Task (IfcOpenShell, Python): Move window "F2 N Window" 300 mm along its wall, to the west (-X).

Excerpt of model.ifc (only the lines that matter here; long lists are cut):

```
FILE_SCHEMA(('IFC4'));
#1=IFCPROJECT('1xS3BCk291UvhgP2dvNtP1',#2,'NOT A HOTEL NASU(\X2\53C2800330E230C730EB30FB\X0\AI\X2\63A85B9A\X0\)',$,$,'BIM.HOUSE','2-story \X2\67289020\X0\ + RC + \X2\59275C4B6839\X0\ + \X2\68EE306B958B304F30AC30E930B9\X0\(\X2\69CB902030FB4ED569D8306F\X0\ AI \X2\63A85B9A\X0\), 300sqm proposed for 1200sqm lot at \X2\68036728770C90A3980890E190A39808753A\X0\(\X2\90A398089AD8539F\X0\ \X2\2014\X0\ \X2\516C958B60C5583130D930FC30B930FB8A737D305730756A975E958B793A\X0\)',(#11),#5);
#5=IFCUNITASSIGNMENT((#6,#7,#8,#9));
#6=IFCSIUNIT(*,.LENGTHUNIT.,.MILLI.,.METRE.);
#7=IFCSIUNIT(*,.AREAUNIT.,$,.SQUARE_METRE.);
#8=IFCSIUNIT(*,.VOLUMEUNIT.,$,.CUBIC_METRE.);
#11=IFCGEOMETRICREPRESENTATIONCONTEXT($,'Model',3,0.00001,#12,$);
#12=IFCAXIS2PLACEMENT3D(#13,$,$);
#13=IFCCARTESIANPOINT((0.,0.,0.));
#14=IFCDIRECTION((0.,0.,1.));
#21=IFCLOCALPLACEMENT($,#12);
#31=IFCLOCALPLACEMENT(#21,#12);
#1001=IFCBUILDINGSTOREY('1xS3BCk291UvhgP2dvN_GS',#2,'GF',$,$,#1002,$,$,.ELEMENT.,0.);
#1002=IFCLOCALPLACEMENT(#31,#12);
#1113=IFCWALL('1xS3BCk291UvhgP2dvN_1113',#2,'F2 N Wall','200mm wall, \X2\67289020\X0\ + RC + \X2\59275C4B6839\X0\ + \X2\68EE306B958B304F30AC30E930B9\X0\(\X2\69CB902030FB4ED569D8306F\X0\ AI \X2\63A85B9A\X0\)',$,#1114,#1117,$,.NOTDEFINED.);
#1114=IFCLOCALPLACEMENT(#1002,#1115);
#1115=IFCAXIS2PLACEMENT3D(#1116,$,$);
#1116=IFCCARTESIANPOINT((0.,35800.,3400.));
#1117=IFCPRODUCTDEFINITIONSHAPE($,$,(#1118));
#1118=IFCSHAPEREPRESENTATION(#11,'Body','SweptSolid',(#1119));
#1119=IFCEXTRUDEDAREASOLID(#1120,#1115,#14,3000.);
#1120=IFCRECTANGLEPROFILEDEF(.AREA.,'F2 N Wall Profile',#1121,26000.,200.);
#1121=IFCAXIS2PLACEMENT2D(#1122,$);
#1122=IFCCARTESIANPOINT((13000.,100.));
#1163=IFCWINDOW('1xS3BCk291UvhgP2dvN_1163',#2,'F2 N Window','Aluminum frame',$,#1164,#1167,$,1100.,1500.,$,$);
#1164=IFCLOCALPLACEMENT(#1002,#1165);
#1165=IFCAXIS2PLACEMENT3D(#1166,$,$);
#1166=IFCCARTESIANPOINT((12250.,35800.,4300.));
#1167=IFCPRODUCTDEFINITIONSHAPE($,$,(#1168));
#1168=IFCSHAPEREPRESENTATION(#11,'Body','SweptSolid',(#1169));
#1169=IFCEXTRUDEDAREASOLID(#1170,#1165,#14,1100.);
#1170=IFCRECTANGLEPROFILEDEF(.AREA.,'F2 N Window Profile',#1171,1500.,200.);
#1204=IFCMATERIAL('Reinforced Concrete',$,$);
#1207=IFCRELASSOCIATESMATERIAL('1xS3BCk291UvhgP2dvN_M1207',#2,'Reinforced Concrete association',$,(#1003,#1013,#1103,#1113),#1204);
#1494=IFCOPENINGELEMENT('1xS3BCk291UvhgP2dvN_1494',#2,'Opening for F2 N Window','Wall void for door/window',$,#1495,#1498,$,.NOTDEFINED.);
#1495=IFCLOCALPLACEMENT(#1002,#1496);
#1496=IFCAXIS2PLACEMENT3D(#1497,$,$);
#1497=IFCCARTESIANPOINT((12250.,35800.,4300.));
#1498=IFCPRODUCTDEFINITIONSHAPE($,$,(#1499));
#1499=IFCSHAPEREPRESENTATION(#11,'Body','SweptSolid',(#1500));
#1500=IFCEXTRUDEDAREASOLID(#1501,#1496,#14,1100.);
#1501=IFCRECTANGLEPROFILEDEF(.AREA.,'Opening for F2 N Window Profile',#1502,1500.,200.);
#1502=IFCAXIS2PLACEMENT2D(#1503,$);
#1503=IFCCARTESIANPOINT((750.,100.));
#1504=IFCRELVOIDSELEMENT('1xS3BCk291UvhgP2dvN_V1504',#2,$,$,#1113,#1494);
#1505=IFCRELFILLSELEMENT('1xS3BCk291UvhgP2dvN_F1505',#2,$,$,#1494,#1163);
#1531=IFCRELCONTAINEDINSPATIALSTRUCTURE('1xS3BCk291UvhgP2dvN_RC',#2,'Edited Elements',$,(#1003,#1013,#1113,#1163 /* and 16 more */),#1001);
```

```python
import ifcopenshell
import ifcopenshell.api.geometry
import ifcopenshell.util.placement
import ifcopenshell.util.unit

model = ifcopenshell.open("model.ifc")
unit_scale = ifcopenshell.util.unit.calculate_unit_scale(model)

window = model.by_guid("1xS3BCk291UvhgP2dvN_1163")
opening = window.FillsVoids[0].RelatingOpeningElement
wall = opening.VoidsElements[0].RelatingBuildingElement

wall_matrix = ifcopenshell.util.placement.get_local_placement(wall.ObjectPlacement)
shift = wall_matrix[:3, 0] * -0.3 / unit_scale
before = ifcopenshell.util.placement.get_local_placement(window.ObjectPlacement)[:3, 3].copy()

# The window is not placed relative to its opening, so move both.
for product in (opening, window):
    matrix = ifcopenshell.util.placement.get_local_placement(product.ObjectPlacement)
    matrix[:3, 3] += shift
    ifcopenshell.api.geometry.edit_object_placement(model, product=product, matrix=matrix, is_si=False)

after = ifcopenshell.util.placement.get_local_placement(window.ObjectPlacement)[:3, 3]
print("window moved by", (after - before).round(3) + 0.0)

model.write("model-out.ifc")
```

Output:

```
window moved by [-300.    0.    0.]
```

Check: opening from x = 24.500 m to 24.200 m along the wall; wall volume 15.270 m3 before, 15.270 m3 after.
